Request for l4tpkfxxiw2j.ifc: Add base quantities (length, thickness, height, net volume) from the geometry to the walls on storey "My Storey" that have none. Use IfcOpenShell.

First a look at what the model holds.

```python
import ifcopenshell
import ifcopenshell.util.element
import ifcopenshell.util.unit

model = ifcopenshell.open("l4tpkfxxiw2j.ifc")
print(model.schema)
for unit_type in ("LENGTHUNIT", "AREAUNIT", "VOLUMEUNIT"):
    print(unit_type, ifcopenshell.util.unit.calculate_unit_scale(model, unit_type))
storey = next(s for s in model.by_type("IfcBuildingStorey") if s.Name == "My Storey")
walls = [e for e in ifcopenshell.util.element.get_decomposition(storey) if e.is_a("IfcWall")]
for e in sorted(walls, key=lambda e: e.id()):
    print(e.id(), e.is_a(), e.Name, list(ifcopenshell.util.element.get_psets(e, qtos_only=True)), sep=" | ")
```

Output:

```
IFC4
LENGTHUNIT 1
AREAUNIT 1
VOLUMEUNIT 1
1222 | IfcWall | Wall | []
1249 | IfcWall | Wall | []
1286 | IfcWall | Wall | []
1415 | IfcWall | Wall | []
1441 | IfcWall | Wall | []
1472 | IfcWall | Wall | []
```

```python
import ifcopenshell
import ifcopenshell.api.pset
import ifcopenshell.geom
import ifcopenshell.util.element
import ifcopenshell.util.shape
import ifcopenshell.util.unit

model = ifcopenshell.open("l4tpkfxxiw2j.ifc")
unit_scale = ifcopenshell.util.unit.calculate_unit_scale(model)
volume_scale = ifcopenshell.util.unit.calculate_unit_scale(model, "VOLUMEUNIT")
settings = ifcopenshell.geom.settings()

storey = next(s for s in model.by_type("IfcBuildingStorey") if s.Name == "My Storey")
walls = [e for e in ifcopenshell.util.element.get_decomposition(storey) if e.is_a("IfcWall")]

for e in sorted(walls, key=lambda e: e.id()):
    if ifcopenshell.util.element.get_psets(e, qtos_only=True, should_inherit=False):
        continue
    # Geometry comes back in metres, in the element's own axes.
    shape = ifcopenshell.geom.create_shape(settings, e)
    values = {
        "Length": ifcopenshell.util.shape.get_x(shape.geometry) / unit_scale,
        "Width": ifcopenshell.util.shape.get_y(shape.geometry) / unit_scale,
        "Height": ifcopenshell.util.shape.get_z(shape.geometry) / unit_scale,
        "NetVolume": ifcopenshell.util.shape.get_volume(shape.geometry) / volume_scale,
    }
    qto = ifcopenshell.api.pset.add_qto(model, product=e, name="Qto_WallBaseQuantities")
    ifcopenshell.api.pset.edit_qto(model, qto=qto, properties=values)
    print(e.id(), {k: round(v, 3) for k, v in values.items()})

model.write("l4tpkfxxiw2j_v2.ifc")
```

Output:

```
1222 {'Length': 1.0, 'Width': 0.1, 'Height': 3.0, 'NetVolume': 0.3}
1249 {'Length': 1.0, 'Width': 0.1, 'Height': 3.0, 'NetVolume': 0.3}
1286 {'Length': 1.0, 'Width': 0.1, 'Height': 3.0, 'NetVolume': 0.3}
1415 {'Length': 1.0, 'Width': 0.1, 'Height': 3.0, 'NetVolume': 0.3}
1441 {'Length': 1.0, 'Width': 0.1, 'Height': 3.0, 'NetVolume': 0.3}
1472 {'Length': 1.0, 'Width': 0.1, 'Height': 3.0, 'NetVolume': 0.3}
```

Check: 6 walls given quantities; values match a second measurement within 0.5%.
